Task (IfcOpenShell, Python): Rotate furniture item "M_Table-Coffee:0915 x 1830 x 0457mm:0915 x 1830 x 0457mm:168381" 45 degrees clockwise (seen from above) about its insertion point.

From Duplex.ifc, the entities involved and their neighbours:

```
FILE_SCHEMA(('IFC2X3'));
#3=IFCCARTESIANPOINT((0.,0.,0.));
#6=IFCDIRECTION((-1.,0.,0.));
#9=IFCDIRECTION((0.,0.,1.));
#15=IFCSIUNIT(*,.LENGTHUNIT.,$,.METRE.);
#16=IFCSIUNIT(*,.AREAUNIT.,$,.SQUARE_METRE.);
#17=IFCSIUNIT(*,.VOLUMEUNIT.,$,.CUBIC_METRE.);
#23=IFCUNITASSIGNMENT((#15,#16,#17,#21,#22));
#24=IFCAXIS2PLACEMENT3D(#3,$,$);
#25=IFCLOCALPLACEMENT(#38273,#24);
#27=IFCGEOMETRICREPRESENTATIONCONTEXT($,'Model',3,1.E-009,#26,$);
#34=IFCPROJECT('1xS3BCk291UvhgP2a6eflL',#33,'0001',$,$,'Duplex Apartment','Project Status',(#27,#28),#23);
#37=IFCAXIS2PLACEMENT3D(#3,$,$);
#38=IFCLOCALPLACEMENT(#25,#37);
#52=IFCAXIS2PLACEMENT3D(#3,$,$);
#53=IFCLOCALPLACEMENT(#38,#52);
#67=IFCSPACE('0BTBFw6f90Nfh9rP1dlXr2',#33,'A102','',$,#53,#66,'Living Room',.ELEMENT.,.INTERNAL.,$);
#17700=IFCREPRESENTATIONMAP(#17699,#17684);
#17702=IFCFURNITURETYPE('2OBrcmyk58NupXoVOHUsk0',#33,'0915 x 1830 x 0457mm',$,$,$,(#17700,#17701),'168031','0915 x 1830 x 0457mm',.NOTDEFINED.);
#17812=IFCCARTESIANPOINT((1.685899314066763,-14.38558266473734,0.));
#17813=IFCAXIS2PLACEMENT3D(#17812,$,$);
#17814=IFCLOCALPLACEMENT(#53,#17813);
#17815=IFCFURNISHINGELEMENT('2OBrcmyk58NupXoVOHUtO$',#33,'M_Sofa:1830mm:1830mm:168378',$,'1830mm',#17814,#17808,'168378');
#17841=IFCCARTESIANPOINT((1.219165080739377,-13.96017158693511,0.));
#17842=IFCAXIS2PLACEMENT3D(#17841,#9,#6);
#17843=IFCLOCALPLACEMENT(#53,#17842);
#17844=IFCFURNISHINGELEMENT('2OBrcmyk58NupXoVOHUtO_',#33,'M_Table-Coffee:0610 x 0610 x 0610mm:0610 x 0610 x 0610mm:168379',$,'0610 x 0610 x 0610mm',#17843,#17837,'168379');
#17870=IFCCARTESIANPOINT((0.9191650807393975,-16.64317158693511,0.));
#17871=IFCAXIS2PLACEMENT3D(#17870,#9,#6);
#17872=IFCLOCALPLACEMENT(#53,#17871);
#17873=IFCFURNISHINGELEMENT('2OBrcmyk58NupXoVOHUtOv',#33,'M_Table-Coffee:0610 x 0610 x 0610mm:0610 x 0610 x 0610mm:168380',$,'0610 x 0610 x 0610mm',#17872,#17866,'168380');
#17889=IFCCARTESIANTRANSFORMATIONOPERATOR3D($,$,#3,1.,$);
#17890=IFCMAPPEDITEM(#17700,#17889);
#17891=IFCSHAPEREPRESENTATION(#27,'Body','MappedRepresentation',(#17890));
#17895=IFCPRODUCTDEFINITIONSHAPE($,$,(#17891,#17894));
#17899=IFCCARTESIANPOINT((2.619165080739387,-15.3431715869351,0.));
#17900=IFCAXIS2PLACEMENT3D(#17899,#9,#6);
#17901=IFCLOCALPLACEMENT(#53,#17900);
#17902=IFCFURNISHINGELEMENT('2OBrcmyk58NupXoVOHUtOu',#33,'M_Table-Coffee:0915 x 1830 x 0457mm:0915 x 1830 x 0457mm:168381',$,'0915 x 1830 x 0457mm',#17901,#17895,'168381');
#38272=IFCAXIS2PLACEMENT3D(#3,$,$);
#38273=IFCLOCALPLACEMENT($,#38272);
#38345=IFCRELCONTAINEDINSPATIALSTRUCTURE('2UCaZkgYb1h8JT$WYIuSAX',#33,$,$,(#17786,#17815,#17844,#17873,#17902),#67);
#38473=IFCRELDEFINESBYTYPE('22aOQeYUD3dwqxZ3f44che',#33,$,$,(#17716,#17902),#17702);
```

```python
import ifcopenshell
import ifcopenshell.api.geometry
import ifcopenshell.util.placement

model = ifcopenshell.open("Duplex.ifc")

item = model.by_guid("2OBrcmyk58NupXoVOHUtOu")
matrix = ifcopenshell.util.placement.get_local_placement(item.ObjectPlacement)
matrix = matrix @ ifcopenshell.util.placement.rotation(-45, "Z")
ifcopenshell.api.geometry.edit_object_placement(model, product=item, matrix=matrix, is_si=False)

print(ifcopenshell.util.placement.get_local_placement(item.ObjectPlacement).round(3) + 0.0)

model.write("Duplex_v2.ifc")
```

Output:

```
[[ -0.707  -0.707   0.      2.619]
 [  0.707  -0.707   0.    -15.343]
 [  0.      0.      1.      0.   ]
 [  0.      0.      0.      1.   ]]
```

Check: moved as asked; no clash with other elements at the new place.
